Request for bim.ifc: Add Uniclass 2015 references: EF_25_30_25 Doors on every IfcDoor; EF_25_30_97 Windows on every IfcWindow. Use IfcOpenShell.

First a look at what the model holds.

```python
import ifcopenshell

model = ifcopenshell.open("bim.ifc")
print(model.schema)
print("classifications:", [c.Name for c in model.by_type("IfcClassification")])
for ifc_class in ("IfcDoor", "IfcRoof", "IfcStair", "IfcWall", "IfcWindow"):
    print(ifc_class, len(model.by_type(ifc_class)))
```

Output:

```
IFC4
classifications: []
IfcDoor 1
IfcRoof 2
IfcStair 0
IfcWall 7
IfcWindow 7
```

```python
import ifcopenshell
import ifcopenshell.api.classification

model = ifcopenshell.open("bim.ifc")

system = ifcopenshell.api.classification.add_classification(model, classification="Uniclass 2015")

codes = {
    "IfcDoor": ("EF_25_30_25", "Doors"),
    "IfcWindow": ("EF_25_30_97", "Windows"),
}
for ifc_class, (code, name) in codes.items():
    products = model.by_type(ifc_class)
    ifcopenshell.api.classification.add_reference(
        model, products=products, classification=system, identification=code, name=name
    )
    print(code, len(products))

model.write("bim_rev.ifc")
```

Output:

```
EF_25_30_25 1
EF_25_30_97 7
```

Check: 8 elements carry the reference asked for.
